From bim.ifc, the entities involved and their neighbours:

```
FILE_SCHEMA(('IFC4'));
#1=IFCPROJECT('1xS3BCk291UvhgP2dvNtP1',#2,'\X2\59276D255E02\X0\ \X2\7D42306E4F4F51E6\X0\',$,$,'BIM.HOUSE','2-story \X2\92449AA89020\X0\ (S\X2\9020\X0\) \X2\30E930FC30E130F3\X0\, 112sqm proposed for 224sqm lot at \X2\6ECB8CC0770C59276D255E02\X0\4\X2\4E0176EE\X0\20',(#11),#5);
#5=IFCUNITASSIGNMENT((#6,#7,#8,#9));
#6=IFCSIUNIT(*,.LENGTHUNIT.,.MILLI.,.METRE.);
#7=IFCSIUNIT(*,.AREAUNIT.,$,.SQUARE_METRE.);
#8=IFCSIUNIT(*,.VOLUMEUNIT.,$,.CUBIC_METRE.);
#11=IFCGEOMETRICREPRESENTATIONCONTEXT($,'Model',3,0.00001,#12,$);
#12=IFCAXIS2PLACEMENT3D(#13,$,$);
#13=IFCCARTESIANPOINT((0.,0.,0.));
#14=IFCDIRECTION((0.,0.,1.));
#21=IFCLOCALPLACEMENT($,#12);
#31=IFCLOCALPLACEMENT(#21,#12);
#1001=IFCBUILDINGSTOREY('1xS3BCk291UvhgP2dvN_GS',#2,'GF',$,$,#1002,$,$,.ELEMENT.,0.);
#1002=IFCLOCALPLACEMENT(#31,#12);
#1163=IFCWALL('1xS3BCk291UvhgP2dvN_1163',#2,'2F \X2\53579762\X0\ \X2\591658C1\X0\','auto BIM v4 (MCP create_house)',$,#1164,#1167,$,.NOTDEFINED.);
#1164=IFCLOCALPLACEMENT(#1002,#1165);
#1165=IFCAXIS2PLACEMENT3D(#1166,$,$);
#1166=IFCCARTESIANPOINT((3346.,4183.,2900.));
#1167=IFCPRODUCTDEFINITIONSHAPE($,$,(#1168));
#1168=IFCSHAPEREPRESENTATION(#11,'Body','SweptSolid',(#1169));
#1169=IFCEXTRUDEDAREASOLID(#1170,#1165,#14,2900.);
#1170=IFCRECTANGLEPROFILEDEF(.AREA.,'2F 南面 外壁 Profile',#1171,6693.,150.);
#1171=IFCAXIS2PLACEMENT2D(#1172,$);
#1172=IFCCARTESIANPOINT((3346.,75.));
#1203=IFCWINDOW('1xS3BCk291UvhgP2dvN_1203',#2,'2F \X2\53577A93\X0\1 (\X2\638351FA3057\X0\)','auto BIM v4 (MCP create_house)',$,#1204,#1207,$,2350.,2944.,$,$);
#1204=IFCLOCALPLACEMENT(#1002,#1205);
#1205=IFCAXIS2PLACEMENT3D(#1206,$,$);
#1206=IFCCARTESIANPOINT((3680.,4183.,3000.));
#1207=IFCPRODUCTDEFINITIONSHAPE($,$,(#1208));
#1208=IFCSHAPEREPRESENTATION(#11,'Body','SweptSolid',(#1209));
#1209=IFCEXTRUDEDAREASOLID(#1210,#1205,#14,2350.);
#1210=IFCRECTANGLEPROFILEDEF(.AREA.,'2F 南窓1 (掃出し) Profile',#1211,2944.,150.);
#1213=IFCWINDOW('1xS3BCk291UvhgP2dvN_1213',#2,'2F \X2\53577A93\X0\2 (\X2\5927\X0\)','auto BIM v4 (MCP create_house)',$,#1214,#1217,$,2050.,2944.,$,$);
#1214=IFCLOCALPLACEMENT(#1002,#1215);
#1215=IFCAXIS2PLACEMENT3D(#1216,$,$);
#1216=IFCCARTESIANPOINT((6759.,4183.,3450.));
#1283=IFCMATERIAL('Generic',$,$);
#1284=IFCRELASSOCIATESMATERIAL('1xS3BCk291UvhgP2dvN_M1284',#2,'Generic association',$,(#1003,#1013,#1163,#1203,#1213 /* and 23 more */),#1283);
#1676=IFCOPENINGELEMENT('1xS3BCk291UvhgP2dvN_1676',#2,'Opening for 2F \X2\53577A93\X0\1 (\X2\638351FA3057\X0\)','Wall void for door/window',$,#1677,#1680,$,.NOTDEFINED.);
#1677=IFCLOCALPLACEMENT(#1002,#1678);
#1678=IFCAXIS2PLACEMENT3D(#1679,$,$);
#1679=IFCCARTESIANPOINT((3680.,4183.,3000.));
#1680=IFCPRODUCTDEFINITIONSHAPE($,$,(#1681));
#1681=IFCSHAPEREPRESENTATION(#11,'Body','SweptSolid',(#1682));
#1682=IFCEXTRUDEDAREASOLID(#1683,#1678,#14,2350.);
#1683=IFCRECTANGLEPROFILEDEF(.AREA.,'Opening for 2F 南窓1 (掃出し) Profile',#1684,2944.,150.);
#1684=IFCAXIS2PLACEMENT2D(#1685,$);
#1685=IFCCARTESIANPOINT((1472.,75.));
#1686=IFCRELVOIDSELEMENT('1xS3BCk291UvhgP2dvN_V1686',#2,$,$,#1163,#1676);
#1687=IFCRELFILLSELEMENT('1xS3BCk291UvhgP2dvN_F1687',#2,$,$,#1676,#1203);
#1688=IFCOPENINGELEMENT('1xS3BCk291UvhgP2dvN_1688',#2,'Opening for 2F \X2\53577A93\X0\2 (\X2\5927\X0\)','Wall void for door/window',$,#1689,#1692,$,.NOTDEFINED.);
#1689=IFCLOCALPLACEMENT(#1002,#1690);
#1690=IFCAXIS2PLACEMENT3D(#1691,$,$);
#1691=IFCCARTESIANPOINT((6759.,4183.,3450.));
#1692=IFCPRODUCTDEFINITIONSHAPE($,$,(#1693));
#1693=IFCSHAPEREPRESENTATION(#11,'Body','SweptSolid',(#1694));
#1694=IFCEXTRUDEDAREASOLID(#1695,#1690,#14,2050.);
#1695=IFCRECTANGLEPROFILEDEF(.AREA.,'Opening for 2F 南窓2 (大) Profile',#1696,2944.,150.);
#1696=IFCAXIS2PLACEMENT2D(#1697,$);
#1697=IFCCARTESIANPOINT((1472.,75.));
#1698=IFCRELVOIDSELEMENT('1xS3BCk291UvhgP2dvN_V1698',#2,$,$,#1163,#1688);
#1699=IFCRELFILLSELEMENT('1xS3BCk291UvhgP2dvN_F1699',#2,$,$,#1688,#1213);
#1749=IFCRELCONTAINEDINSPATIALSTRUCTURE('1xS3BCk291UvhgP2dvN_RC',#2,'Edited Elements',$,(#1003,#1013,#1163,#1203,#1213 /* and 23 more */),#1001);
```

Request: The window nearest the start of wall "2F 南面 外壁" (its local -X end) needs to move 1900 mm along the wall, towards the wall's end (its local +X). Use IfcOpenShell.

```python
import ifcopenshell
import ifcopenshell.api.geometry
import ifcopenshell.util.placement
import ifcopenshell.util.unit

model = ifcopenshell.open("bim.ifc")
unit_scale = ifcopenshell.util.unit.calculate_unit_scale(model)

window = model.by_id(1203)
opening = window.FillsVoids[0].RelatingOpeningElement
wall = opening.VoidsElements[0].RelatingBuildingElement

wall_matrix = ifcopenshell.util.placement.get_local_placement(wall.ObjectPlacement)
shift = wall_matrix[:3, 0] * 1.9 / unit_scale
before = ifcopenshell.util.placement.get_local_placement(window.ObjectPlacement)[:3, 3].copy()

# The window is not placed relative to its opening, so move both.
for product in (opening, window):
    matrix = ifcopenshell.util.placement.get_local_placement(product.ObjectPlacement)
    matrix[:3, 3] += shift
    ifcopenshell.api.geometry.edit_object_placement(model, product=product, matrix=matrix, is_si=False)

after = ifcopenshell.util.placement.get_local_placement(window.ObjectPlacement)[:3, 3]
print("window moved by", (after - before).round(3) + 0.0)

model.write("bim_rev.ifc")
```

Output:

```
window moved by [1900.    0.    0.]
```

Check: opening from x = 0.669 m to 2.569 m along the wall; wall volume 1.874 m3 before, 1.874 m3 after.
